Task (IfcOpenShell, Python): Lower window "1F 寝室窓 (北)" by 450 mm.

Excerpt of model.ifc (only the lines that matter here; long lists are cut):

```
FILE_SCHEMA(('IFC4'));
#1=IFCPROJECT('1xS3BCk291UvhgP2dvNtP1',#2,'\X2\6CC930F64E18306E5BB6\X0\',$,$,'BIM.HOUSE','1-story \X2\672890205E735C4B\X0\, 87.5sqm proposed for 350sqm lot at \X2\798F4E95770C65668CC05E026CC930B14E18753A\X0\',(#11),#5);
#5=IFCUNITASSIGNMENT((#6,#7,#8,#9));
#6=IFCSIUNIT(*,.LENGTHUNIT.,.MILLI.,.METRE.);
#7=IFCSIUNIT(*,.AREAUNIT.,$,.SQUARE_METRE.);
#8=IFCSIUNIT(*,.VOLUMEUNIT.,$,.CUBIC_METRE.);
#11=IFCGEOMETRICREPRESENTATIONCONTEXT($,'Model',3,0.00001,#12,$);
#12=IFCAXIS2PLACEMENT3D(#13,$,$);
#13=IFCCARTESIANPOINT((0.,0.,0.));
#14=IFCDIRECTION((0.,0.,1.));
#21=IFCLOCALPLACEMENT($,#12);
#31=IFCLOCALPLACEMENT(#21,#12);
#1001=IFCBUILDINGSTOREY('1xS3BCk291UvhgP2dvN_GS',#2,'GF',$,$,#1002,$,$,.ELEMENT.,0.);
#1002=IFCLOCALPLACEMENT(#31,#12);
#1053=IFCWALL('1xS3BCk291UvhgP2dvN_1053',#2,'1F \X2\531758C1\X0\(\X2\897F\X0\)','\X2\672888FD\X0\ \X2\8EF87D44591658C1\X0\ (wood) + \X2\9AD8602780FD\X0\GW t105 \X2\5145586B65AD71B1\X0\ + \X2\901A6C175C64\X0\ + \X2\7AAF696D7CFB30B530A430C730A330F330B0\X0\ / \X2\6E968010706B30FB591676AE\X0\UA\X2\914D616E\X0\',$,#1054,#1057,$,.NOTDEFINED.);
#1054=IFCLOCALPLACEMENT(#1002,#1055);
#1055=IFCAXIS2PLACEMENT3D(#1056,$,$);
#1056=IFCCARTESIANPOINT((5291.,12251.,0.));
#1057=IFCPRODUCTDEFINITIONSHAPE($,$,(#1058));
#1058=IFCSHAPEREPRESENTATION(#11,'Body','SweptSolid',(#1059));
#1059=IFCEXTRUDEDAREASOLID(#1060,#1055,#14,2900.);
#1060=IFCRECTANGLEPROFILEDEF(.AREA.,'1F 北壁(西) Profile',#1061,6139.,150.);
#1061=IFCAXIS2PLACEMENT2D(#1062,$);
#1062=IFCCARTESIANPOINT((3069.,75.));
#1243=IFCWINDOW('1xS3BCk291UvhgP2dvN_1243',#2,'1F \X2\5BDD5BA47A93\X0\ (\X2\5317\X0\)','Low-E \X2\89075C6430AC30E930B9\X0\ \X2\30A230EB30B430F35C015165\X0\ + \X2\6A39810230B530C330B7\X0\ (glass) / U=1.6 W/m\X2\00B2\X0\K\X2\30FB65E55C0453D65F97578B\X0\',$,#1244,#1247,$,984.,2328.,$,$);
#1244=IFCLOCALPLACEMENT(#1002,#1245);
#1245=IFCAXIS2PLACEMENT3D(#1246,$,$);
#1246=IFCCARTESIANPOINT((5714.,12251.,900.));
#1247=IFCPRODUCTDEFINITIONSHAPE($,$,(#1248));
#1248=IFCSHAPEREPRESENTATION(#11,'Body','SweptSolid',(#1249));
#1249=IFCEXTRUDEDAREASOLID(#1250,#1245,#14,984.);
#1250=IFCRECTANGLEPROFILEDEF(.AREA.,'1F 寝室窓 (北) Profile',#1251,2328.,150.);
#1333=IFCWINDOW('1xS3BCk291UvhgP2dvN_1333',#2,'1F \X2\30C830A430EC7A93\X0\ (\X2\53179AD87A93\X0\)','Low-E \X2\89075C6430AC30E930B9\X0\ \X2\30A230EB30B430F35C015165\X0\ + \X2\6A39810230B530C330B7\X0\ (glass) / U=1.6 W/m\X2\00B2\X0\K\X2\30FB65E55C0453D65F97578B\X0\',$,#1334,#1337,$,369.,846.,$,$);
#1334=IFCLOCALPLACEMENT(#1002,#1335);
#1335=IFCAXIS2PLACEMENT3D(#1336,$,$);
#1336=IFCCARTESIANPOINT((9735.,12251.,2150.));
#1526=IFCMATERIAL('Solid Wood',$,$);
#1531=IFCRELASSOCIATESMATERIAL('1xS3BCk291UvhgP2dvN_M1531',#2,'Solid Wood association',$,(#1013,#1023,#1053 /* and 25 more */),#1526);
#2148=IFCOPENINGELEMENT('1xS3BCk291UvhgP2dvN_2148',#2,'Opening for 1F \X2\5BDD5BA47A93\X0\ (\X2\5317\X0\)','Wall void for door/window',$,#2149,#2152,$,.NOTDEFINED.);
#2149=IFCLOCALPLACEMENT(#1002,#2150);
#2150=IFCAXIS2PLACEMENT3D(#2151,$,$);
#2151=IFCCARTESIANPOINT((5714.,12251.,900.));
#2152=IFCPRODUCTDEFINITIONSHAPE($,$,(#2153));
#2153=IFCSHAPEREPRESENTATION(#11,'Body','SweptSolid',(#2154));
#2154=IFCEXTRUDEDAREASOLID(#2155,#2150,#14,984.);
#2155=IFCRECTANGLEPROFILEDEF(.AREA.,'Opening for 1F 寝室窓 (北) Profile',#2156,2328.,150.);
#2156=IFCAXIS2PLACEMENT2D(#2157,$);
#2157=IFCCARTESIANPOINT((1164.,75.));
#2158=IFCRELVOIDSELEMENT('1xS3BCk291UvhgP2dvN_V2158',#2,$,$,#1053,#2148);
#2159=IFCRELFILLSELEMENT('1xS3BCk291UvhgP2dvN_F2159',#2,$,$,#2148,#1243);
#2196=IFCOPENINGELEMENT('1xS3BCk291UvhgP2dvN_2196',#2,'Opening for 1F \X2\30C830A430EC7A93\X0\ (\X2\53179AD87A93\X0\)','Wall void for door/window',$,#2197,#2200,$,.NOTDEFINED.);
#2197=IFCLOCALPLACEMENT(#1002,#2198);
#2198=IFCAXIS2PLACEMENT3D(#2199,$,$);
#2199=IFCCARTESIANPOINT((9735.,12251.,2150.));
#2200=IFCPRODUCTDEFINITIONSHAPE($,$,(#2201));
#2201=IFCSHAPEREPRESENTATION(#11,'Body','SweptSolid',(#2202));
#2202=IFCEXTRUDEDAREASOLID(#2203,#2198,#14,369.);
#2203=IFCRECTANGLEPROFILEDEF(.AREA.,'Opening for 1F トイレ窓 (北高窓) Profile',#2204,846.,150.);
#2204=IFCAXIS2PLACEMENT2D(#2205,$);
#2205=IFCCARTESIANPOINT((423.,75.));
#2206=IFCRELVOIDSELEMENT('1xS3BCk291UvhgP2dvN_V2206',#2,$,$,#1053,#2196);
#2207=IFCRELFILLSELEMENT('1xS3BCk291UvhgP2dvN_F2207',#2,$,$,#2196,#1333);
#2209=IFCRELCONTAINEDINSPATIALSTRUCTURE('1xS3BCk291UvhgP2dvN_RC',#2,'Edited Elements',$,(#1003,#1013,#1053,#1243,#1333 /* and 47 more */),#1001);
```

```python
import numpy as np
import ifcopenshell
import ifcopenshell.api.geometry
import ifcopenshell.util.placement
import ifcopenshell.util.unit

model = ifcopenshell.open("model.ifc")
unit_scale = ifcopenshell.util.unit.calculate_unit_scale(model)

window = model.by_guid("1xS3BCk291UvhgP2dvN_1243")
opening = window.FillsVoids[0].RelatingOpeningElement
dz = -0.45 / unit_scale

shift = np.array([0.0, 0.0, dz])
# The window is not placed relative to its opening, so move both.
for product in (opening, window):
    matrix = ifcopenshell.util.placement.get_local_placement(product.ObjectPlacement)
    matrix[:3, 3] += shift
    ifcopenshell.api.geometry.edit_object_placement(model, product=product, matrix=matrix, is_si=False)

print(f"moved by {dz * unit_scale:+.3f} m")

model.write("model_v2.ifc")
```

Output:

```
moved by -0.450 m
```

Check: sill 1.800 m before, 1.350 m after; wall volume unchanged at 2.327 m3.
